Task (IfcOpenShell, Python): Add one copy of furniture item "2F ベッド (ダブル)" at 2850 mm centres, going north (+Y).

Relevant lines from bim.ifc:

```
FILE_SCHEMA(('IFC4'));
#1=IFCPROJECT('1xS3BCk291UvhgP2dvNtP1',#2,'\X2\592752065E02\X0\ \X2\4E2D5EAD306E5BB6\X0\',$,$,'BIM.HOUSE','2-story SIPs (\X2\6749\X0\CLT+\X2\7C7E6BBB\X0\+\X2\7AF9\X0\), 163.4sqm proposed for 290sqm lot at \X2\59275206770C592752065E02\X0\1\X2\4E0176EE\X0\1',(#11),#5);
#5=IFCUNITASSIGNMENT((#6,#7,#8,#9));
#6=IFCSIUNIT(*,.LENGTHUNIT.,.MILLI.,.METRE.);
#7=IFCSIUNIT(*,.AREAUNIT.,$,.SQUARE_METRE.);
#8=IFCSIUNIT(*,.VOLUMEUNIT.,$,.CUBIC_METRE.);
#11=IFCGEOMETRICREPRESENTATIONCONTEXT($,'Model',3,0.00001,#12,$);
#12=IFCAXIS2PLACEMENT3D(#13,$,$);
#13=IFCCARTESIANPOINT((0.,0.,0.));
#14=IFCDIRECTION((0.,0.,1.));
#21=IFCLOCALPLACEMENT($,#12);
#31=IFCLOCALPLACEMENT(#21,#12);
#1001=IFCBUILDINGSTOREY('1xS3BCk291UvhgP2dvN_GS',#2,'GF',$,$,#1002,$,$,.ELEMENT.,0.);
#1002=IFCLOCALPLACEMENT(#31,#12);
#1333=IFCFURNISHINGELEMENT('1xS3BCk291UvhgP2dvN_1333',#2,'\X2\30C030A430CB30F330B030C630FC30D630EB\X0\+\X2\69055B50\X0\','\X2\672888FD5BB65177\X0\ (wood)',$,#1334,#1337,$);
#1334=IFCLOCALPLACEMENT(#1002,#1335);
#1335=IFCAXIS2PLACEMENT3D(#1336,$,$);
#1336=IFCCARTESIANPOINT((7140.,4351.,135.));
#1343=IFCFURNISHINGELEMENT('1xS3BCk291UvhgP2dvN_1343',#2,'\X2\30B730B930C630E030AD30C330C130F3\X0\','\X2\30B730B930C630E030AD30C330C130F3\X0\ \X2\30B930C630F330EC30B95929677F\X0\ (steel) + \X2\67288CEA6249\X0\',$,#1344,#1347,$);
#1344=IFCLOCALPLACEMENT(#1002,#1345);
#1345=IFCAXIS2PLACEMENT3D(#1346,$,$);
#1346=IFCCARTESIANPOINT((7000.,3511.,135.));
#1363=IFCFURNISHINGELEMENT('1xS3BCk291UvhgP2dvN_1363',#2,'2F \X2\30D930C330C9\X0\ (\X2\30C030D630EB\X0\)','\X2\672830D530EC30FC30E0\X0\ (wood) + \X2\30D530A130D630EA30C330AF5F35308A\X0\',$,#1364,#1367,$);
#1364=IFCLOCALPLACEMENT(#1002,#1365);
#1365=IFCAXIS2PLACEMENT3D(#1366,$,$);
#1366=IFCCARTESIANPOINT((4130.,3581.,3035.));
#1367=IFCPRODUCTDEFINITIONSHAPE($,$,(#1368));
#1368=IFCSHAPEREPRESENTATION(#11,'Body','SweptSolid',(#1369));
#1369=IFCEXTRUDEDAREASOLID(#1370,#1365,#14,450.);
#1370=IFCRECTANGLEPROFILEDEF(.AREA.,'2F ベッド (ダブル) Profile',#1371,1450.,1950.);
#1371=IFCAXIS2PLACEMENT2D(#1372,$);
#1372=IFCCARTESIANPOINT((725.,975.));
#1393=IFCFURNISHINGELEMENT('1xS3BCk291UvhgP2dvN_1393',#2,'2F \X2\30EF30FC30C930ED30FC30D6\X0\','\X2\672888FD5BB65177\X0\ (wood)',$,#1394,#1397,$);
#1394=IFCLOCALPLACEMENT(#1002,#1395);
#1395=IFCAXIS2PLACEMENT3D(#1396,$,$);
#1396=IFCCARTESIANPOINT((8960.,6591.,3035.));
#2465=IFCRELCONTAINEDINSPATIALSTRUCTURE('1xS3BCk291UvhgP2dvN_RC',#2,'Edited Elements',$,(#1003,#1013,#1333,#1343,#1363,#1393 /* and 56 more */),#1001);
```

```python
import numpy as np
import ifcopenshell
import ifcopenshell.api.geometry
import ifcopenshell.api.root
import ifcopenshell.util.element
import ifcopenshell.util.placement

model = ifcopenshell.open("bim.ifc")


def reuse_history(source, copy):
    """copy_class also copies each property set's owner history, people and application; keep the originals."""
    for rel in copy.IsDefinedBy:
        if rel.is_a("IfcRelDefinesByProperties") and (history := rel.RelatingPropertyDefinition.OwnerHistory):
            rel.RelatingPropertyDefinition.OwnerHistory = source.OwnerHistory
            ifcopenshell.util.element.remove_deep2(model, history)


source = model.by_guid("1xS3BCk291UvhgP2dvN_1363")
base = ifcopenshell.util.placement.get_local_placement(source.ObjectPlacement)
step = np.array([0.0, 1.0, 0.0]) * 2850.0

for i in range(1, 2):
    copy = ifcopenshell.api.root.copy_class(model, product=source)
    copy.Representation = ifcopenshell.util.element.copy_deep(
        model, source.Representation, exclude=["IfcGeometricRepresentationContext", "IfcRepresentationMap"]
    )
    reuse_history(source, copy)
    matrix = base.copy()
    matrix[:3, 3] += i * step
    print("added at", matrix[:3, 3].round(3) + 0.0)
    ifcopenshell.api.geometry.edit_object_placement(model, product=copy, matrix=matrix, is_si=False)

model.write("bim_edited.ifc")
```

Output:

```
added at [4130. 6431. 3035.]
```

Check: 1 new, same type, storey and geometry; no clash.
